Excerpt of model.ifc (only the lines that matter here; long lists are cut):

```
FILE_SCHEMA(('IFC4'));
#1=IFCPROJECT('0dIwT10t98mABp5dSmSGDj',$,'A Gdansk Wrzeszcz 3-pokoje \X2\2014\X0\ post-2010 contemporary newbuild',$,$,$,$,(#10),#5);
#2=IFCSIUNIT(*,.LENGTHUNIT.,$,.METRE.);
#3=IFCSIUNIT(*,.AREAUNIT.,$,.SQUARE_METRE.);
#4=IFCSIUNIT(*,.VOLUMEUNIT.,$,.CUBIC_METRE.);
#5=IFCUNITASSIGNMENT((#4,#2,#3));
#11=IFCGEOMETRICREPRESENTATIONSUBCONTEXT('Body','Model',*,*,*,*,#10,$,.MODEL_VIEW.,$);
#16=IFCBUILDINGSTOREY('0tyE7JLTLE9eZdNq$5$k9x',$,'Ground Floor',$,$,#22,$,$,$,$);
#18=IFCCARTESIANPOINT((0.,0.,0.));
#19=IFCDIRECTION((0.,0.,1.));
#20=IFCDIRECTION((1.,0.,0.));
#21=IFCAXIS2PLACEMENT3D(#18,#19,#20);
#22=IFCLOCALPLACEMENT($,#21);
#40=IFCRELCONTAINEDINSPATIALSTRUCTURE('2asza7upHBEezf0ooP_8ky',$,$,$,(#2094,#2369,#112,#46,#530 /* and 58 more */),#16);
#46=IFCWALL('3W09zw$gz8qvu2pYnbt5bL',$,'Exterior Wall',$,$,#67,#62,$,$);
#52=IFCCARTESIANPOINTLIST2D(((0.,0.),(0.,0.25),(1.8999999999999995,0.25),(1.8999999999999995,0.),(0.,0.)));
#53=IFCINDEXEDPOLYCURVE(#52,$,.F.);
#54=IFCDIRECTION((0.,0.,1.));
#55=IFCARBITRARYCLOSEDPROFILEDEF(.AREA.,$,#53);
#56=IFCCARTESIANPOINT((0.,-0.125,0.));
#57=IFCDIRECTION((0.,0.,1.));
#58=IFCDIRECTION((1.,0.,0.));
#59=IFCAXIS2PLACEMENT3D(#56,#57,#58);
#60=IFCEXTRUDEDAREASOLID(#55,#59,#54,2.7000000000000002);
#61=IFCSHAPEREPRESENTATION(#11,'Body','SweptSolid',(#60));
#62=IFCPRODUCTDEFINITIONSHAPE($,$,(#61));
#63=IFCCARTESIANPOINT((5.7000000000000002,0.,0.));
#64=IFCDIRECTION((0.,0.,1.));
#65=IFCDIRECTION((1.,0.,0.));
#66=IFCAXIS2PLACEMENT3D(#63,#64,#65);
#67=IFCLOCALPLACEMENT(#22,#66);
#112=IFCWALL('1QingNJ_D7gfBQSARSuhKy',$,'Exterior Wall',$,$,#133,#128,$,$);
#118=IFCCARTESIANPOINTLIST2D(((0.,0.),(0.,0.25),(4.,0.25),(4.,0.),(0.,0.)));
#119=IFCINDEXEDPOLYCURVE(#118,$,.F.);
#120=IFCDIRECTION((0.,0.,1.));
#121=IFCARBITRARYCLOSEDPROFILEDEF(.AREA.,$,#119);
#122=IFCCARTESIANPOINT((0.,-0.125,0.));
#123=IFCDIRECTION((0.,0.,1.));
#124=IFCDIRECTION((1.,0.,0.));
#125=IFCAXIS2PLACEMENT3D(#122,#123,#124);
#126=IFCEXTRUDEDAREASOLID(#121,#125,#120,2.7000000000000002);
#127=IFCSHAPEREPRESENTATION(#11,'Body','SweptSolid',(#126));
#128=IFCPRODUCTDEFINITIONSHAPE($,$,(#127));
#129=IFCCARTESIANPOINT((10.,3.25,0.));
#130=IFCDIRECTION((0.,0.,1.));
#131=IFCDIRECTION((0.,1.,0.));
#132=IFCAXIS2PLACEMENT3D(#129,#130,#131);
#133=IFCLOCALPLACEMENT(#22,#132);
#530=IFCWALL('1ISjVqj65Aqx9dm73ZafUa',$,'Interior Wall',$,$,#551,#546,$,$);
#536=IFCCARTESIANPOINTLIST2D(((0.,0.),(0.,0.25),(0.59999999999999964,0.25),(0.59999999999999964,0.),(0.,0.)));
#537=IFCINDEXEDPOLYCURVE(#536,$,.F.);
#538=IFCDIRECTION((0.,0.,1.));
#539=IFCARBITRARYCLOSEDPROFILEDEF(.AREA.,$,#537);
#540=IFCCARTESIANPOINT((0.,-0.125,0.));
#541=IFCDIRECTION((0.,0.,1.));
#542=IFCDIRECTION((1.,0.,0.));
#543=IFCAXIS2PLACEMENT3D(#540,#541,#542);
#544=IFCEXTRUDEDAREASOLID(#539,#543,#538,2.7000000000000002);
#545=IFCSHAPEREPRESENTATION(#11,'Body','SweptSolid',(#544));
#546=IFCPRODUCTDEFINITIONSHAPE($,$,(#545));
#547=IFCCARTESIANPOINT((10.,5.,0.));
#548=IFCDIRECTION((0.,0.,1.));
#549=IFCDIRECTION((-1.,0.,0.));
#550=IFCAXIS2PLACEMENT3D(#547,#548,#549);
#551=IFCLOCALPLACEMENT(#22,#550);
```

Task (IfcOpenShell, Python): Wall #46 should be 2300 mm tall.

```python
import ifcopenshell
import ifcopenshell.geom
import ifcopenshell.util.representation
import ifcopenshell.util.shape

model = ifcopenshell.open("model.ifc")
settings = ifcopenshell.geom.settings()


def volume(element):
    """Net volume in cubic metres, openings subtracted."""
    shape = ifcopenshell.geom.create_shape(settings, element)
    return ifcopenshell.util.shape.get_volume(shape.geometry)


wall = model.by_id(46)
before = volume(wall)

body = ifcopenshell.util.representation.get_representation(wall, "Model", "Body")
solid = body.Items[0]
old_height = solid.Depth
solid.Depth = 2.3
after = volume(wall)

print(f"height {old_height:g} -> {solid.Depth:g}, volume {before:.3f} -> {after:.3f} m3")

model.write("model_edited.ifc")
```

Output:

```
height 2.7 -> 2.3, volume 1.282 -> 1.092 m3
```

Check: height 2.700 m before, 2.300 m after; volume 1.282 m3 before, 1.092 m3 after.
